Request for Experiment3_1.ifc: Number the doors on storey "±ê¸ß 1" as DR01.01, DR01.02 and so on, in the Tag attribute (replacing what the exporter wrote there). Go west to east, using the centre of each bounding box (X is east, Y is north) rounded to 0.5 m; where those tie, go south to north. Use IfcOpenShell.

First a look at what the model holds.

```python
import ifcopenshell
import ifcopenshell.util.element
import ifcopenshell.util.placement

model = ifcopenshell.open("Experiment3_1.ifc")
print(model.schema)
storey = next(s for s in model.by_type("IfcBuildingStorey") if s.Name == "±ê¸ß 1")
doors = [e for e in ifcopenshell.util.element.get_decomposition(storey) if e.is_a("IfcDoor")]
for e in sorted(doors, key=lambda e: e.id()):
    origin = ifcopenshell.util.placement.get_local_placement(e.ObjectPlacement)[:3, 3]
    print(e.id(), e.Tag, e.Name, origin.round(2) + 0.0, sep=" | ")
```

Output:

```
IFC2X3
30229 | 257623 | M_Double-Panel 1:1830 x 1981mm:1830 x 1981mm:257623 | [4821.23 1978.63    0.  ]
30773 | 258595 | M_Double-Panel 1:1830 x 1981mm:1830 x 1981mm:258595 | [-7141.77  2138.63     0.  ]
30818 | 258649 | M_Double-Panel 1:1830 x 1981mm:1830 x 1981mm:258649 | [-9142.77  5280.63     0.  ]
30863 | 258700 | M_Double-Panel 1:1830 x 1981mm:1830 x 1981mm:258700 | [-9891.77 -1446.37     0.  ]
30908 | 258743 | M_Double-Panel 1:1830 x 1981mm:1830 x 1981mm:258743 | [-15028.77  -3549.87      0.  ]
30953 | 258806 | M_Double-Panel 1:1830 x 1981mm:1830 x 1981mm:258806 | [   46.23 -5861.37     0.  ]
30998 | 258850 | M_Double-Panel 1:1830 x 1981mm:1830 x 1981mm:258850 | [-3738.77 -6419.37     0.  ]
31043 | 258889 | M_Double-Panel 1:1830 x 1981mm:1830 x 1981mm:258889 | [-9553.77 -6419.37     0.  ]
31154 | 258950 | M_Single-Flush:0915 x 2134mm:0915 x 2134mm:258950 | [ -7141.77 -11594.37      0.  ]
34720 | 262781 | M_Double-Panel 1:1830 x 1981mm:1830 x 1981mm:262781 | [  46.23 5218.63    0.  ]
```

```python
import ifcopenshell
import ifcopenshell.geom
import ifcopenshell.util.element
import ifcopenshell.util.shape

model = ifcopenshell.open("Experiment3_1.ifc")
settings = ifcopenshell.geom.settings()
settings.set("use-world-coords", True)


def centre(element):
    shape = ifcopenshell.geom.create_shape(settings, element)
    return ifcopenshell.util.shape.get_bbox_centroid(shape.geometry)


storey = next(s for s in model.by_type("IfcBuildingStorey") if s.Name == "±ê¸ß 1")
doors = [e for e in ifcopenshell.util.element.get_decomposition(storey) if e.is_a("IfcDoor")]

# Insertion points can sit at a corner or the storey origin, so sort by the geometry (in metres).
centres = {e: centre(e) for e in doors}
doors.sort(key=lambda e: (round(centres[e][0] / 0.5), centres[e][1]))

for i, e in enumerate(doors, start=1):
    number = f"DR01.{i:02d}"
    e.Tag = number
    print(e.id(), number)

model.write("Experiment3_1_rev.ifc")
```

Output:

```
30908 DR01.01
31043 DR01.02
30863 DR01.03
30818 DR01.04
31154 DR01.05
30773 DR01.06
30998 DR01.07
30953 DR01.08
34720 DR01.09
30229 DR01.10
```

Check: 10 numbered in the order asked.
